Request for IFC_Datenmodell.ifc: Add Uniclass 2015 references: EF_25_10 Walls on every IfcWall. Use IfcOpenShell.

First a look at what the model holds.

```python
import ifcopenshell

model = ifcopenshell.open("IFC_Datenmodell.ifc")
print(model.schema)
print("classifications:", [c.Name for c in model.by_type("IfcClassification")])
for ifc_class in ("IfcDoor", "IfcRoof", "IfcStair", "IfcWall", "IfcWindow"):
    print(ifc_class, len(model.by_type(ifc_class)))
```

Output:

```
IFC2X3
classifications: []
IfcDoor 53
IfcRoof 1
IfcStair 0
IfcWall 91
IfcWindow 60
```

```python
import ifcopenshell
import ifcopenshell.api.classification

model = ifcopenshell.open("IFC_Datenmodell.ifc")

# IFC2X3 requires Source and Edition and has no link from the project to the system.
system = model.create_entity("IfcClassification", Source="NBS", Edition="2015", Name="Uniclass 2015")

codes = {
    "IfcWall": ("EF_25_10", "Walls"),
}
for ifc_class, (code, name) in codes.items():
    products = model.by_type(ifc_class)
    ifcopenshell.api.classification.add_reference(
        model, products=products, classification=system, identification=code, name=name
    )
    print(code, len(products))

model.write("IFC_Datenmodell_v2.ifc")
```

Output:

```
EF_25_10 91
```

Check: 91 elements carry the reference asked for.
